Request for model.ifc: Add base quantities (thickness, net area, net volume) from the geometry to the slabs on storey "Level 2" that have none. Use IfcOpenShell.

First a look at what the model holds.

```python
import ifcopenshell
import ifcopenshell.util.element
import ifcopenshell.util.unit

model = ifcopenshell.open("model.ifc")
print(model.schema)
for unit_type in ("LENGTHUNIT", "AREAUNIT", "VOLUMEUNIT"):
    print(unit_type, ifcopenshell.util.unit.calculate_unit_scale(model, unit_type))
storey = next(s for s in model.by_type("IfcBuildingStorey") if s.Name == "Level 2")
slabs = [e for e in ifcopenshell.util.element.get_decomposition(storey) if e.is_a("IfcSlab")]
for e in sorted(slabs, key=lambda e: e.id()):
    print(e.id(), e.is_a(), e.Name, list(ifcopenshell.util.element.get_psets(e, qtos_only=True)), sep=" | ")
```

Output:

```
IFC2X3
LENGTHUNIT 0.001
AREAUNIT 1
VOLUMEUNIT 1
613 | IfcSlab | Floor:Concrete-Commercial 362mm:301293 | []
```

```python
import ifcopenshell
import ifcopenshell.api.pset
import ifcopenshell.geom
import ifcopenshell.util.element
import ifcopenshell.util.shape
import ifcopenshell.util.unit

model = ifcopenshell.open("model.ifc")
unit_scale = ifcopenshell.util.unit.calculate_unit_scale(model)
area_scale = ifcopenshell.util.unit.calculate_unit_scale(model, "AREAUNIT")
volume_scale = ifcopenshell.util.unit.calculate_unit_scale(model, "VOLUMEUNIT")
settings = ifcopenshell.geom.settings()

storey = next(s for s in model.by_type("IfcBuildingStorey") if s.Name == "Level 2")
slabs = [e for e in ifcopenshell.util.element.get_decomposition(storey) if e.is_a("IfcSlab")]

for e in sorted(slabs, key=lambda e: e.id()):
    if ifcopenshell.util.element.get_psets(e, qtos_only=True, should_inherit=False):
        continue
    # Geometry comes back in metres, in the element's own axes.
    shape = ifcopenshell.geom.create_shape(settings, e)
    values = {
        "Width": ifcopenshell.util.shape.get_z(shape.geometry) / unit_scale,
        "NetArea": ifcopenshell.util.shape.get_footprint_area(shape.geometry) / area_scale,
        "NetVolume": ifcopenshell.util.shape.get_volume(shape.geometry) / volume_scale,
    }
    qto = ifcopenshell.api.pset.add_qto(model, product=e, name="BaseQuantities")
    ifcopenshell.api.pset.edit_qto(model, qto=qto, properties=values)
    print(e.id(), {k: round(v, 3) for k, v in values.items()})

model.write("model_edited.ifc")
```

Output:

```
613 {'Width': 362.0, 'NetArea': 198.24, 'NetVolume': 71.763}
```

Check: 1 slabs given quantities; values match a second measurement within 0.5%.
